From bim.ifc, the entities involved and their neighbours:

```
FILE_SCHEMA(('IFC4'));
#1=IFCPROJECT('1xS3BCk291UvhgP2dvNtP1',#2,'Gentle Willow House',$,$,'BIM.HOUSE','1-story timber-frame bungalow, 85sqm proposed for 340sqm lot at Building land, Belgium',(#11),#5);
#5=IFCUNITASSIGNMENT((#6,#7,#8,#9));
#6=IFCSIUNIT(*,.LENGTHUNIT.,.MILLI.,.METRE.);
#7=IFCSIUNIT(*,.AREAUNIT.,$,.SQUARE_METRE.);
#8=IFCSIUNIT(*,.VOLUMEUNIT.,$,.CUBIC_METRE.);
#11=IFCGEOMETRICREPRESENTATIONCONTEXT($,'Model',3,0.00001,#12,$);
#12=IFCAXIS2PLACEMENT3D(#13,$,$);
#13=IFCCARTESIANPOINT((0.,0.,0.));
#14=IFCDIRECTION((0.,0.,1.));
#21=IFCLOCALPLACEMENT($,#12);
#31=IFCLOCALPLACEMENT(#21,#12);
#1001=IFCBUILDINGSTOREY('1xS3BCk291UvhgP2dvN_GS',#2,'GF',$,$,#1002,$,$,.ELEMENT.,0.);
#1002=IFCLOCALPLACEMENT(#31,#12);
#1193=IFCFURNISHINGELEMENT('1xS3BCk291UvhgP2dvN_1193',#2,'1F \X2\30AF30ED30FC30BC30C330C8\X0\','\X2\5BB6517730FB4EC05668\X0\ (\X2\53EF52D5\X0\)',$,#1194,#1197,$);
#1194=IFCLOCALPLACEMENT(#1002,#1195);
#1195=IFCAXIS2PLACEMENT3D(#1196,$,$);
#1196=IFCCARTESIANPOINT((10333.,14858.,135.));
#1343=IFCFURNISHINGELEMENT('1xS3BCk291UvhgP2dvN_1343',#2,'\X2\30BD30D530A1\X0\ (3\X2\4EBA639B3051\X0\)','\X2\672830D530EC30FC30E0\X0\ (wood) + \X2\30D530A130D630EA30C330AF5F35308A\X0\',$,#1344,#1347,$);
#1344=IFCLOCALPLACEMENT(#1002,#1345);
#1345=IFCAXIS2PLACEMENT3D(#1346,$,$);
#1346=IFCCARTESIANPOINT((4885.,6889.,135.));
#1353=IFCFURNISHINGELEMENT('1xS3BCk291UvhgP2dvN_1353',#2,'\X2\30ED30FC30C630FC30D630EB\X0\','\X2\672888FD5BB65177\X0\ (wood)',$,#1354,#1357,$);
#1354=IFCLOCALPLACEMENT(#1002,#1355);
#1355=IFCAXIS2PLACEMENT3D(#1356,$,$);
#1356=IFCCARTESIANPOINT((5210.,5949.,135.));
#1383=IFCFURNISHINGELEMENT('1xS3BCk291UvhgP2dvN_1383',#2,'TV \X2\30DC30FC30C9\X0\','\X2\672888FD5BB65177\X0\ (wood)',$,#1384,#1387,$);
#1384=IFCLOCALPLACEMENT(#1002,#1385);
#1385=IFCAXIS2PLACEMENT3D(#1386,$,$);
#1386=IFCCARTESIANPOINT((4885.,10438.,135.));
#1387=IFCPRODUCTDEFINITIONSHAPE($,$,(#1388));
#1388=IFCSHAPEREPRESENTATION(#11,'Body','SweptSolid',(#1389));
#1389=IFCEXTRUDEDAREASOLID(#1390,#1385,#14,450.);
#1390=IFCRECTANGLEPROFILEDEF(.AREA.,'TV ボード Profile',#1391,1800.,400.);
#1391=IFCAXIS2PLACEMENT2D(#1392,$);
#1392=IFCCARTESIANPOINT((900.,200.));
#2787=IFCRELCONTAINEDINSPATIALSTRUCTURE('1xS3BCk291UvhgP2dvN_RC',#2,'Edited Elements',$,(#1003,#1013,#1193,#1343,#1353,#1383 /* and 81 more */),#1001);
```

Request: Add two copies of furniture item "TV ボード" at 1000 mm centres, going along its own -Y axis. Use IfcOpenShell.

```python
import ifcopenshell
import ifcopenshell.api.geometry
import ifcopenshell.api.root
import ifcopenshell.util.element
import ifcopenshell.util.placement
import ifcopenshell.util.unit

model = ifcopenshell.open("bim.ifc")
unit_scale = ifcopenshell.util.unit.calculate_unit_scale(model)


def reuse_history(source, copy):
    """copy_class also copies each property set's owner history, people and application; keep the originals."""
    for rel in copy.IsDefinedBy:
        if rel.is_a("IfcRelDefinesByProperties") and (history := rel.RelatingPropertyDefinition.OwnerHistory):
            rel.RelatingPropertyDefinition.OwnerHistory = source.OwnerHistory
            ifcopenshell.util.element.remove_deep2(model, history)


source = model.by_guid("1xS3BCk291UvhgP2dvN_1383")
base = ifcopenshell.util.placement.get_local_placement(source.ObjectPlacement)
step = -base[:3, 1] * 1 / unit_scale

for i in range(1, 3):
    copy = ifcopenshell.api.root.copy_class(model, product=source)
    copy.Representation = ifcopenshell.util.element.copy_deep(
        model, source.Representation, exclude=["IfcGeometricRepresentationContext", "IfcRepresentationMap"]
    )
    reuse_history(source, copy)
    matrix = base.copy()
    matrix[:3, 3] += i * step
    print("added at", matrix[:3, 3].round(3) + 0.0)
    ifcopenshell.api.geometry.edit_object_placement(model, product=copy, matrix=matrix, is_si=False)

model.write("bim_edited.ifc")
```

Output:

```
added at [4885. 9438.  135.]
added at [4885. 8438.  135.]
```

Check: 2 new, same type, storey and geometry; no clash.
